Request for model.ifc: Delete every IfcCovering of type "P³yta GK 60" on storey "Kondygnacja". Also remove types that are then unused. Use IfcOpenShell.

First a look at what the model holds.

```python
import ifcopenshell
import ifcopenshell.util.element

model = ifcopenshell.open("model.ifc")
print(model.schema)
storey = next(s for s in model.by_type("IfcBuildingStorey") if s.Name == "Kondygnacja")
coverings = [e for e in ifcopenshell.util.element.get_decomposition(storey) if e.is_a("IfcCovering")]
seen = {}
for e in coverings:
    element_type = ifcopenshell.util.element.get_type(e)
    name = element_type.Name if element_type not in (None, e) else None
    seen[name] = seen.get(name, 0) + 1
for name, count in sorted(seen.items(), key=str):
    print(count, "x", name)
```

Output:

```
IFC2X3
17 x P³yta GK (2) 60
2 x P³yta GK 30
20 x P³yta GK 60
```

```python
import ifcopenshell
import ifcopenshell.api.root
import ifcopenshell.util.element

model = ifcopenshell.open("model.ifc")

storey = next(s for s in model.by_type("IfcBuildingStorey") if s.Name == "Kondygnacja")
coverings = [e for e in ifcopenshell.util.element.get_decomposition(storey) if e.is_a("IfcCovering")]
targets = [e for e in coverings if (t := ifcopenshell.util.element.get_type(e)) not in (None, e) and t.Name == "P³yta GK 60"]
types = {ifcopenshell.util.element.get_type(e) for e in targets} - {None, *targets}

for e in targets:
    ifcopenshell.api.root.remove_product(model, product=e)
print(len(targets), "removed")

unused = [t for t in types if not ifcopenshell.util.element.get_types(t)]
for t in unused:
    ifcopenshell.api.root.remove_product(model, product=t)
print(len(unused), "unused types removed")

model.write("model_updated.ifc")
```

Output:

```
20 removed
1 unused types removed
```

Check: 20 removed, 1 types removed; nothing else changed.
